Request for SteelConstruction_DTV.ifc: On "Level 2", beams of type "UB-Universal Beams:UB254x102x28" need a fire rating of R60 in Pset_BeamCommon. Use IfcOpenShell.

First a look at what the model holds.

```python
import ifcopenshell
import ifcopenshell.util.element

model = ifcopenshell.open("SteelConstruction_DTV.ifc")
print(model.schema)
storey = next(s for s in model.by_type("IfcBuildingStorey") if s.Name == "Level 2")
beams = [e for e in ifcopenshell.util.element.get_decomposition(storey) if e.is_a("IfcBeam")]
seen = {}
for e in beams:
    element_type = ifcopenshell.util.element.get_type(e)
    key = (element_type.Name if element_type != e and element_type else None, ifcopenshell.util.element.get_pset(e, "Pset_BeamCommon", "FireRating"))
    seen[key] = seen.get(key, 0) + 1
for (name, value), count in sorted(seen.items(), key=str):
    print(count, "x", name, "|", value)
```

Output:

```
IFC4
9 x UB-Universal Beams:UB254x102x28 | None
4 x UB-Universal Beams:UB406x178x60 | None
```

```python
import ifcopenshell
import ifcopenshell.api.pset
import ifcopenshell.util.element

model = ifcopenshell.open("SteelConstruction_DTV.ifc")

storey = next(s for s in model.by_type("IfcBuildingStorey") if s.Name == "Level 2")
beams = [e for e in ifcopenshell.util.element.get_decomposition(storey) if e.is_a("IfcBeam")]

count = 0
for e in beams:
    element_type = ifcopenshell.util.element.get_type(e)
    if element_type in (None, e) or element_type.Name != "UB-Universal Beams:UB254x102x28":
        continue
    # add_pset returns the element's existing set when there is one.
    pset = ifcopenshell.api.pset.add_pset(model, product=e, name="Pset_BeamCommon")
    ifcopenshell.api.pset.edit_pset(model, pset=pset, properties={"FireRating": "R60"})
    count += 1

print(count, "beams updated")

model.write("SteelConstruction_DTV_v2.ifc")
```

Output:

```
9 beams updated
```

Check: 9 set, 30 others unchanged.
